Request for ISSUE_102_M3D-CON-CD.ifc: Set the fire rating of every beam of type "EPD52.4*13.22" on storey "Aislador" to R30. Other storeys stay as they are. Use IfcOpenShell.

First a look at what the model holds.

```python
import ifcopenshell
import ifcopenshell.util.element

model = ifcopenshell.open("ISSUE_102_M3D-CON-CD.ifc")
print(model.schema)
storey = next(s for s in model.by_type("IfcBuildingStorey") if s.Name == "Aislador")
beams = [e for e in ifcopenshell.util.element.get_decomposition(storey) if e.is_a("IfcBeam")]
seen = {}
for e in beams:
    element_type = ifcopenshell.util.element.get_type(e)
    key = (element_type.Name if element_type != e and element_type else None, ifcopenshell.util.element.get_pset(e, "Pset_BeamCommon", "FireRating"))
    seen[key] = seen.get(key, 0) + 1
for (name, value), count in sorted(seen.items(), key=str):
    print(count, "x", name, "|", value)
```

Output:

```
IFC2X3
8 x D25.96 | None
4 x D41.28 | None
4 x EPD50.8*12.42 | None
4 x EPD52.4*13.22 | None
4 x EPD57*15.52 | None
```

```python
import ifcopenshell
import ifcopenshell.api.pset
import ifcopenshell.util.element

model = ifcopenshell.open("ISSUE_102_M3D-CON-CD.ifc")

storey = next(s for s in model.by_type("IfcBuildingStorey") if s.Name == "Aislador")
beams = [e for e in ifcopenshell.util.element.get_decomposition(storey) if e.is_a("IfcBeam")]

count = 0
for e in beams:
    element_type = ifcopenshell.util.element.get_type(e)
    if element_type in (None, e) or element_type.Name != "EPD52.4*13.22":
        continue
    found = ifcopenshell.util.element.get_pset(e, "Pset_BeamCommon", should_inherit=False)
    if found:
        pset = model.by_id(found["id"])
        if len(ifcopenshell.util.element.get_elements_by_pset(pset)) > 1:
            pset = ifcopenshell.api.pset.unshare_pset(model, products=[e], pset=pset)[0]
    else:
        pset = ifcopenshell.api.pset.add_pset(model, product=e, name="Pset_BeamCommon")
    ifcopenshell.api.pset.edit_pset(model, pset=pset, properties={"FireRating": "R30"})
    count += 1

print(count, "beams updated")

model.write("ISSUE_102_M3D-CON-CD_updated.ifc")
```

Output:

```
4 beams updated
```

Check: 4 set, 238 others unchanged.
